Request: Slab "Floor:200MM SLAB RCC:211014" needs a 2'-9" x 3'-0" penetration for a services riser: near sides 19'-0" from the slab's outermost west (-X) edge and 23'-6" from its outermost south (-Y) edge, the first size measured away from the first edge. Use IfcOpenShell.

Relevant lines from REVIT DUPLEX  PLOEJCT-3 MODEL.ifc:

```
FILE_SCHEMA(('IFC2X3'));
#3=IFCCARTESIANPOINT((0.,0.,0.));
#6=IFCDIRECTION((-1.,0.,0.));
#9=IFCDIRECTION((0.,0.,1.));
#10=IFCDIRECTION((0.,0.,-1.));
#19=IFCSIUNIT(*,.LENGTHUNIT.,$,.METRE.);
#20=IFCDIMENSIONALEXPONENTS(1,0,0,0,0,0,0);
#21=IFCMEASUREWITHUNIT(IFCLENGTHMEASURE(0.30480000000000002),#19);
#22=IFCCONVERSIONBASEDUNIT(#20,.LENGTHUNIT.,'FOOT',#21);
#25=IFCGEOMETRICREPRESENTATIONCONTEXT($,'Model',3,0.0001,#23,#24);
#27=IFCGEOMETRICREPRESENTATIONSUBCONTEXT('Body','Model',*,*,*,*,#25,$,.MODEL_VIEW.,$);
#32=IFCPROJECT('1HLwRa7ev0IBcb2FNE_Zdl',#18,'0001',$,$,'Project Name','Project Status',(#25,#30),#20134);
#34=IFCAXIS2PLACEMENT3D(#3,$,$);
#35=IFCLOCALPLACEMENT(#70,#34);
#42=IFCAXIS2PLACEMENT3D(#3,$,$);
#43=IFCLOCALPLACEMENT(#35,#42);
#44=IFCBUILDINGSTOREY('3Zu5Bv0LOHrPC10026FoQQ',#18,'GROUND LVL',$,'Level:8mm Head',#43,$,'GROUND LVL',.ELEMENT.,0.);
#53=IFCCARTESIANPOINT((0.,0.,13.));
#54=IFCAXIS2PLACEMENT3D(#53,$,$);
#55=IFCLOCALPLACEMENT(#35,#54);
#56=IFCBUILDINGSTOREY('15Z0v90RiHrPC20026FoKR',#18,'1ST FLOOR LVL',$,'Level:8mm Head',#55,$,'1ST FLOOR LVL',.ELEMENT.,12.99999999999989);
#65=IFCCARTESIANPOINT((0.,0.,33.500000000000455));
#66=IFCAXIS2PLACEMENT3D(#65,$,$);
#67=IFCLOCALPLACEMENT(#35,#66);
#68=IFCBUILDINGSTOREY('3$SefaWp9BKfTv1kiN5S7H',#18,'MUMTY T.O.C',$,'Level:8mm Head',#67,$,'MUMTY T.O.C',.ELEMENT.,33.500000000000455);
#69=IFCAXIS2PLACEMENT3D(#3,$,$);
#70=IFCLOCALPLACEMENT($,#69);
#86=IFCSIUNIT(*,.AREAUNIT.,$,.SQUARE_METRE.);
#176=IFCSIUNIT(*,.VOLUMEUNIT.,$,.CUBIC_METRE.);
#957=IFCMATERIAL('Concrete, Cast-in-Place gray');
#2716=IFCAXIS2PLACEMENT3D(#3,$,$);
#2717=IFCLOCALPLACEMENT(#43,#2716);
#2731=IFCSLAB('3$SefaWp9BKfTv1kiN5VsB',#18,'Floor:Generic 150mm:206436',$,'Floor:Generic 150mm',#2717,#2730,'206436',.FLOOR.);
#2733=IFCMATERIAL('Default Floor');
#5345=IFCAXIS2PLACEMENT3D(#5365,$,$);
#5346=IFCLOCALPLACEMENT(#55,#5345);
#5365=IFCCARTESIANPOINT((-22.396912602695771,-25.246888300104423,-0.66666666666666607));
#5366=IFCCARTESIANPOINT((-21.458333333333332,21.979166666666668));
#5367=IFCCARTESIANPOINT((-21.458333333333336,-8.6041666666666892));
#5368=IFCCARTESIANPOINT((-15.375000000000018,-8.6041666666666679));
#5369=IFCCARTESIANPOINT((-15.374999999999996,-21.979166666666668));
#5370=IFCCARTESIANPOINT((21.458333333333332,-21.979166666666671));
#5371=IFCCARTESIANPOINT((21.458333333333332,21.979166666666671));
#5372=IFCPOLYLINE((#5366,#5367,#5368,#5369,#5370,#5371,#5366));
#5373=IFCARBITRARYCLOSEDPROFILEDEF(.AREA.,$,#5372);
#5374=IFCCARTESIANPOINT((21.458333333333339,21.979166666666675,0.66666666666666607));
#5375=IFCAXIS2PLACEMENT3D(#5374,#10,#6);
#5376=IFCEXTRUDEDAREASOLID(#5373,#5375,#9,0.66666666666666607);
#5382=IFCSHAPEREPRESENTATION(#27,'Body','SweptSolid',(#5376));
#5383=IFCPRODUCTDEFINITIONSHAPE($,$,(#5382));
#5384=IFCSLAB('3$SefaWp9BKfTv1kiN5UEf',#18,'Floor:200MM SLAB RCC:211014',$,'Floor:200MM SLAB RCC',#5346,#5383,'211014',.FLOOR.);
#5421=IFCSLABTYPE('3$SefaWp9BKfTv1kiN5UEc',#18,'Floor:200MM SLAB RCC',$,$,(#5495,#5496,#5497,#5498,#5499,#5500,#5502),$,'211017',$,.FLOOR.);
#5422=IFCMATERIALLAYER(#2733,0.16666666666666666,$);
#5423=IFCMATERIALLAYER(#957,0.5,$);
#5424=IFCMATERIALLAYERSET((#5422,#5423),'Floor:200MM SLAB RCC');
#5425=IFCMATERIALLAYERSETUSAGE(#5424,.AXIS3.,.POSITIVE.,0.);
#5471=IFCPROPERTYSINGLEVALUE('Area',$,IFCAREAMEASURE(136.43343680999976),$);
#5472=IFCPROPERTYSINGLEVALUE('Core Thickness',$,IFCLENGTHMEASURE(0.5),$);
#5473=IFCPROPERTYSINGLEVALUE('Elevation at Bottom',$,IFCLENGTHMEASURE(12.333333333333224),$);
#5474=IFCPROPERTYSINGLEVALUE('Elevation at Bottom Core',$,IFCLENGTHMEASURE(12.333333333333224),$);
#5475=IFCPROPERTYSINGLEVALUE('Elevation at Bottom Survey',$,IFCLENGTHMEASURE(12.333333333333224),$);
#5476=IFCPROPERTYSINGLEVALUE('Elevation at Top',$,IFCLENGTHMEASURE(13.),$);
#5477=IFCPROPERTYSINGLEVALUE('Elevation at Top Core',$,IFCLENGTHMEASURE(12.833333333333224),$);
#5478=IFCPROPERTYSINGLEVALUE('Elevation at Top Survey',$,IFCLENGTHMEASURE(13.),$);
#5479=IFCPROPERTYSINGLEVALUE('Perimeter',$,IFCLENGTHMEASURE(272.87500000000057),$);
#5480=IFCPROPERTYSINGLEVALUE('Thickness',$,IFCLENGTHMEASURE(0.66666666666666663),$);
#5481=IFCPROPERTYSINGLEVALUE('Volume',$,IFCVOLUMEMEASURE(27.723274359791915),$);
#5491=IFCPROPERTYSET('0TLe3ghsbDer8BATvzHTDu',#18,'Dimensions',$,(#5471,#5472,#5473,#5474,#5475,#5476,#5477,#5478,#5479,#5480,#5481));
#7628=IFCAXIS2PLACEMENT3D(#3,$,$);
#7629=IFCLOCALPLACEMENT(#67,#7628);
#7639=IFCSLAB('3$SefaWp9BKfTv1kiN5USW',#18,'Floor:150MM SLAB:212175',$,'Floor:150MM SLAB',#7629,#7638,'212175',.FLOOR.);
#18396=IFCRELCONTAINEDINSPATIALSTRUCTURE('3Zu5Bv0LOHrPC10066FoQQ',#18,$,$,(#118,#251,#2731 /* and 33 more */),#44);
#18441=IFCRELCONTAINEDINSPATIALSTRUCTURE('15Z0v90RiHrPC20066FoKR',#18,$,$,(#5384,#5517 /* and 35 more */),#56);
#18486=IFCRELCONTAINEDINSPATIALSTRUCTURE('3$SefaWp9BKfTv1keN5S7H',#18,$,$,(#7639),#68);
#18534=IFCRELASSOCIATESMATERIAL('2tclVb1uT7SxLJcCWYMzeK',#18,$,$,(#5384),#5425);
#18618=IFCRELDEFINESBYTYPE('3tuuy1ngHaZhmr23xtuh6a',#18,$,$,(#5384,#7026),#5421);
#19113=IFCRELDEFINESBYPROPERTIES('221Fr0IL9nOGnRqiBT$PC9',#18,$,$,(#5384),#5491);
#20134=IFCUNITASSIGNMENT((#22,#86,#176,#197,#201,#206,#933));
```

```python
import numpy as np
import ifcopenshell
import ifcopenshell.api.feature
import ifcopenshell.api.geometry
import ifcopenshell.api.pset
import ifcopenshell.api.root
import ifcopenshell.geom
import ifcopenshell.util.element
import ifcopenshell.util.placement
import ifcopenshell.util.representation
import ifcopenshell.util.shape
import ifcopenshell.util.unit

model = ifcopenshell.open("REVIT DUPLEX  PLOEJCT-3 MODEL.ifc")
unit_scale = ifcopenshell.util.unit.calculate_unit_scale(model)
area_scale = ifcopenshell.util.unit.calculate_unit_scale(model, "AREAUNIT")
volume_scale = ifcopenshell.util.unit.calculate_unit_scale(model, "VOLUMEUNIT")
settings = ifcopenshell.geom.settings()


def volume(element):
    """Net volume in cubic metres, openings subtracted."""
    shape = ifcopenshell.geom.create_shape(settings, element)
    return ifcopenshell.util.shape.get_volume(shape.geometry)


slab = model.by_guid("3$SefaWp9BKfTv1kiN5UEf")
before = volume(slab)

# Extent in the slab's own axes, in metres. The edges named are its -X and -Y sides.
slab_shape = ifcopenshell.geom.create_shape(settings, slab)
vertices = ifcopenshell.util.shape.get_vertices(slab_shape.geometry)
x_min, y_min, bottom = vertices.min(axis=0)
top = vertices[:, 2].max()

opening = ifcopenshell.api.root.create_entity(model, ifc_class="IfcOpeningElement", name="Services riser opening")
context = ifcopenshell.util.representation.get_context(model, "Model", "Body", "MODEL_VIEW")
width, depth = 0.8382, 0.9144
outline = [(0.0, 0.0), (width, 0.0), (width, depth), (0.0, depth), (0.0, 0.0)]
# Overshoot both faces by 50 mm so the cut is clean.
shape = ifcopenshell.api.geometry.add_slab_representation(
    model, context=context, depth=top - bottom + 0.1, polyline=outline
)
ifcopenshell.api.geometry.assign_representation(model, product=opening, representation=shape)

matrix = ifcopenshell.util.placement.get_local_placement(slab.ObjectPlacement)
matrix[:, 3] = matrix @ np.append(np.array([x_min + 5.7912, y_min + 7.1628, bottom - 0.05]) / unit_scale, 1.0)
ifcopenshell.api.geometry.edit_object_placement(model, product=opening, matrix=matrix, is_si=False)
ifcopenshell.api.feature.add_feature(model, feature=opening, element=slab)

after = volume(slab)

# Update the slab's stored quantities.
pset = model.by_id(ifcopenshell.util.element.get_pset(slab, "Dimensions", should_inherit=False)["id"])
ifcopenshell.api.pset.edit_pset(model, pset=pset, properties={
    "Area": model.create_entity("IfcAreaMeasure", after / (top - bottom) / area_scale),
    "Volume": model.create_entity("IfcVolumeMeasure", after / volume_scale),
})

print(f"slab volume {before:.3f} -> {after:.3f} m3")

model.write("REVIT DUPLEX  PLOEJCT-3 MODEL_updated.ifc")
```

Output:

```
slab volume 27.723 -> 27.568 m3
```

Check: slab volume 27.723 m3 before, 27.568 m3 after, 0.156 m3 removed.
